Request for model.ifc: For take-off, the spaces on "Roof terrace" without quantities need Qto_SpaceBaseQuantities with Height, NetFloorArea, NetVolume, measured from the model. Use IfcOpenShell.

First a look at what the model holds.

```python
import ifcopenshell
import ifcopenshell.util.element
import ifcopenshell.util.unit

model = ifcopenshell.open("model.ifc")
print(model.schema)
for unit_type in ("LENGTHUNIT", "AREAUNIT", "VOLUMEUNIT"):
    print(unit_type, ifcopenshell.util.unit.calculate_unit_scale(model, unit_type))
storey = next(s for s in model.by_type("IfcBuildingStorey") if s.Name == "Roof terrace")
spaces = [e for e in ifcopenshell.util.element.get_decomposition(storey) if e.is_a("IfcSpace")]
for e in sorted(spaces, key=lambda e: e.id()):
    print(e.id(), e.is_a(), e.Name, list(ifcopenshell.util.element.get_psets(e, qtos_only=True)), sep=" | ")
```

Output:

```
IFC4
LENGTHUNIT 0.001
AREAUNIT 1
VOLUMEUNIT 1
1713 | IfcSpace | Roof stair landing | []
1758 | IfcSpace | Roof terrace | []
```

```python
import ifcopenshell
import ifcopenshell.api.pset
import ifcopenshell.geom
import ifcopenshell.util.element
import ifcopenshell.util.shape
import ifcopenshell.util.unit

model = ifcopenshell.open("model.ifc")
unit_scale = ifcopenshell.util.unit.calculate_unit_scale(model)
area_scale = ifcopenshell.util.unit.calculate_unit_scale(model, "AREAUNIT")
volume_scale = ifcopenshell.util.unit.calculate_unit_scale(model, "VOLUMEUNIT")
settings = ifcopenshell.geom.settings()

storey = next(s for s in model.by_type("IfcBuildingStorey") if s.Name == "Roof terrace")
spaces = [e for e in ifcopenshell.util.element.get_decomposition(storey) if e.is_a("IfcSpace")]

for e in sorted(spaces, key=lambda e: e.id()):
    if ifcopenshell.util.element.get_psets(e, qtos_only=True, should_inherit=False):
        continue
    # Geometry comes back in metres, in the element's own axes.
    shape = ifcopenshell.geom.create_shape(settings, e)
    values = {
        "Height": ifcopenshell.util.shape.get_z(shape.geometry) / unit_scale,
        "NetFloorArea": ifcopenshell.util.shape.get_footprint_area(shape.geometry) / area_scale,
        "NetVolume": ifcopenshell.util.shape.get_volume(shape.geometry) / volume_scale,
    }
    qto = ifcopenshell.api.pset.add_qto(model, product=e, name="Qto_SpaceBaseQuantities")
    ifcopenshell.api.pset.edit_qto(model, qto=qto, properties=values)
    print(e.id(), {k: round(v, 3) for k, v in values.items()})

model.write("model_v2.ifc")
```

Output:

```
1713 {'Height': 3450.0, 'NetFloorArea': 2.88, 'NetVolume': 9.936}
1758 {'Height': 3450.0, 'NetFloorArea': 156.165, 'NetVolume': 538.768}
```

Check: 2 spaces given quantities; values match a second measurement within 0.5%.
